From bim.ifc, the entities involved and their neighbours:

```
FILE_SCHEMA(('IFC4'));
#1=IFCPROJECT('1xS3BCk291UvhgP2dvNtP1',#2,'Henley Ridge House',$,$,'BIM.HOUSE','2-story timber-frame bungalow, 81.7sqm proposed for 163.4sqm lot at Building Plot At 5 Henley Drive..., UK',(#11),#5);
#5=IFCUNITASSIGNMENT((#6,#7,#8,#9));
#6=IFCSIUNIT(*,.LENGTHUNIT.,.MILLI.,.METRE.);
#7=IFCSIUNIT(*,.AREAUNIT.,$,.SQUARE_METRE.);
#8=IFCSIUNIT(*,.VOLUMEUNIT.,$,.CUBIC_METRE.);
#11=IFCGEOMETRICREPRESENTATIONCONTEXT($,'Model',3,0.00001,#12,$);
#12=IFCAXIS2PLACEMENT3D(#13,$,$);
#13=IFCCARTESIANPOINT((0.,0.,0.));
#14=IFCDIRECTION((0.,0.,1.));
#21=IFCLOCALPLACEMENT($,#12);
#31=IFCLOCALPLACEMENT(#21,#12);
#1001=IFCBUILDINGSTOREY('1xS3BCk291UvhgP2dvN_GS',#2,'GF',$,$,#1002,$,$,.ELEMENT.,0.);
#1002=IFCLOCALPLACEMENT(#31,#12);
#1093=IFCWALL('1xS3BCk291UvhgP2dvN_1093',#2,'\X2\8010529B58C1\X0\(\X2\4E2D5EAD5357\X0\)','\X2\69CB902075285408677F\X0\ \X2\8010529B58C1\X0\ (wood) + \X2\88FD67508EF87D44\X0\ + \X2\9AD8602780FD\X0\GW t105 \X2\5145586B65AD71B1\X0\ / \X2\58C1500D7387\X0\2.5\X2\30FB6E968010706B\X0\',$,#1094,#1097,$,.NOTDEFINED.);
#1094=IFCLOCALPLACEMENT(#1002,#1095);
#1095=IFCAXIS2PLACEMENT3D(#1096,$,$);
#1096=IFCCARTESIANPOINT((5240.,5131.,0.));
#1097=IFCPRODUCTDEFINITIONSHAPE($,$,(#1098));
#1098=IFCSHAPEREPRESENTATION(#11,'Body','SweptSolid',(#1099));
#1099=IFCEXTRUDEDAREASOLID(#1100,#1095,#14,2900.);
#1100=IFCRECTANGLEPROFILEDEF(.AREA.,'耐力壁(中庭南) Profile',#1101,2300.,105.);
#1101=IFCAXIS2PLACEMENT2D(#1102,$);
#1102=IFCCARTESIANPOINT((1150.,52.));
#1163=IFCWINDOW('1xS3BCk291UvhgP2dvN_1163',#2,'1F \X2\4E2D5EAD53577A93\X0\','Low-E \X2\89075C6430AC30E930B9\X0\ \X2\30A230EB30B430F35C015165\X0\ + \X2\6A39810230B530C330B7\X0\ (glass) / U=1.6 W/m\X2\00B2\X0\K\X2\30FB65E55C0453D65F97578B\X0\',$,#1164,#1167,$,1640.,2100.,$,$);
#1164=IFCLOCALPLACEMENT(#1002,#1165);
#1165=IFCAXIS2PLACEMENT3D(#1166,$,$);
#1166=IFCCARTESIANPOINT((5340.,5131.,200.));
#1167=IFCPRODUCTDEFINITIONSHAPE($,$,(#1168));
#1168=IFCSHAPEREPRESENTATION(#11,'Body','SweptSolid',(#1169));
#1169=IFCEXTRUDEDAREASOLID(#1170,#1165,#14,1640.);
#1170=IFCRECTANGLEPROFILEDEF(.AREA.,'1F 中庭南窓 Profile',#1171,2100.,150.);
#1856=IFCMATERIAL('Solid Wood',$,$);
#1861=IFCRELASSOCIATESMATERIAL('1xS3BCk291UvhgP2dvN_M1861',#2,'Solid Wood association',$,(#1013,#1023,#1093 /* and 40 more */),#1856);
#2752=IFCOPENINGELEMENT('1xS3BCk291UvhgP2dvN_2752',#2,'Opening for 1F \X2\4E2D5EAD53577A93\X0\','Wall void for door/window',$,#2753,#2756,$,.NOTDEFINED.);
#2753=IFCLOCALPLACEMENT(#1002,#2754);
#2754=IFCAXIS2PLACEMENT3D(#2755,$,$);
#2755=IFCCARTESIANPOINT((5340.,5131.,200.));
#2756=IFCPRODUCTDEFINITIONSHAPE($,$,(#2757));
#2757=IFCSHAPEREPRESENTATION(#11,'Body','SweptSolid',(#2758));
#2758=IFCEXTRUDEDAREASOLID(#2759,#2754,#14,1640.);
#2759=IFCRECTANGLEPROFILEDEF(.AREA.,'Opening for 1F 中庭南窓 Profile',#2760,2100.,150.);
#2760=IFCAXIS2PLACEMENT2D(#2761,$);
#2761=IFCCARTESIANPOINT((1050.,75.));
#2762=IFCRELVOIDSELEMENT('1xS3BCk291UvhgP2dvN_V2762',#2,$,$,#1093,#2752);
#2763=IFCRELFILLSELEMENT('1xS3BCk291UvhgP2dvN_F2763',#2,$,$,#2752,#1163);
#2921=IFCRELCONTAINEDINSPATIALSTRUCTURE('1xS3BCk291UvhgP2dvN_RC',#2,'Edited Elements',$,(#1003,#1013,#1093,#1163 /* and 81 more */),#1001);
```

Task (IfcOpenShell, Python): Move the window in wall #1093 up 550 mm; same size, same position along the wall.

```python
import numpy as np
import ifcopenshell
import ifcopenshell.api.geometry
import ifcopenshell.util.placement
import ifcopenshell.util.unit

model = ifcopenshell.open("bim.ifc")
unit_scale = ifcopenshell.util.unit.calculate_unit_scale(model)

window = model.by_id(1163)
opening = window.FillsVoids[0].RelatingOpeningElement
dz = 0.55 / unit_scale

shift = np.array([0.0, 0.0, dz])
# The window is not placed relative to its opening, so move both.
for product in (opening, window):
    matrix = ifcopenshell.util.placement.get_local_placement(product.ObjectPlacement)
    matrix[:3, 3] += shift
    ifcopenshell.api.geometry.edit_object_placement(model, product=product, matrix=matrix, is_si=False)

print(f"moved by {dz * unit_scale:+.3f} m")

model.write("bim_rev.ifc")
```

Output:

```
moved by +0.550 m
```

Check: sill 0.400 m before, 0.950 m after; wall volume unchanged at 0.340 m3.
